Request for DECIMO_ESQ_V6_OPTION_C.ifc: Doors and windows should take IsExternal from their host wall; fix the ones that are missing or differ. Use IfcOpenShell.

First a look at what the model holds.

```python
import ifcopenshell
import ifcopenshell.util.element

model = ifcopenshell.open("DECIMO_ESQ_V6_OPTION_C.ifc")
print(model.schema)
seen = {}
for e in model.by_type("IfcDoor") + model.by_type("IfcWindow"):
    if not e.FillsVoids:
        continue
    host = e.FillsVoids[0].RelatingOpeningElement.VoidsElements[0].RelatingBuildingElement
    own = ifcopenshell.util.element.get_pset(e, f"Pset_{e.is_a()[3:].removesuffix('StandardCase')}Common", "IsExternal")
    wall = ifcopenshell.util.element.get_pset(host, "Pset_WallCommon", "IsExternal")
    seen[e.is_a(), own, wall] = seen.get((e.is_a(), own, wall), 0) + 1
for (cls, own, wall), count in sorted(seen.items(), key=str):
    print(count, cls, "IsExternal:", own, "| host wall:", wall)
```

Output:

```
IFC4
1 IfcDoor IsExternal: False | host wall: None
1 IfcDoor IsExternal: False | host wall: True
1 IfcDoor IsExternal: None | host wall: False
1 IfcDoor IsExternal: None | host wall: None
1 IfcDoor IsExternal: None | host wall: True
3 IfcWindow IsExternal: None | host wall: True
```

```python
import ifcopenshell
import ifcopenshell.api.pset
import ifcopenshell.util.element

model = ifcopenshell.open("DECIMO_ESQ_V6_OPTION_C.ifc")

count = 0
for ifc_class, pset_name in (("IfcDoor", "Pset_DoorCommon"), ("IfcWindow", "Pset_WindowCommon")):
    for e in model.by_type(ifc_class):
        if not e.FillsVoids:
            continue
        host = e.FillsVoids[0].RelatingOpeningElement.VoidsElements[0].RelatingBuildingElement
        external = ifcopenshell.util.element.get_pset(host, "Pset_WallCommon", "IsExternal")
        if external is None or ifcopenshell.util.element.get_pset(e, pset_name, "IsExternal") == external:
            continue
        pset = ifcopenshell.api.pset.add_pset(model, product=e, name=pset_name)
        ifcopenshell.api.pset.edit_pset(model, pset=pset, properties={"IsExternal": external})
        count += 1

print(count, "updated")

model.write("DECIMO_ESQ_V6_OPTION_C_rev.ifc")
```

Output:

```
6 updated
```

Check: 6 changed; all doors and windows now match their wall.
